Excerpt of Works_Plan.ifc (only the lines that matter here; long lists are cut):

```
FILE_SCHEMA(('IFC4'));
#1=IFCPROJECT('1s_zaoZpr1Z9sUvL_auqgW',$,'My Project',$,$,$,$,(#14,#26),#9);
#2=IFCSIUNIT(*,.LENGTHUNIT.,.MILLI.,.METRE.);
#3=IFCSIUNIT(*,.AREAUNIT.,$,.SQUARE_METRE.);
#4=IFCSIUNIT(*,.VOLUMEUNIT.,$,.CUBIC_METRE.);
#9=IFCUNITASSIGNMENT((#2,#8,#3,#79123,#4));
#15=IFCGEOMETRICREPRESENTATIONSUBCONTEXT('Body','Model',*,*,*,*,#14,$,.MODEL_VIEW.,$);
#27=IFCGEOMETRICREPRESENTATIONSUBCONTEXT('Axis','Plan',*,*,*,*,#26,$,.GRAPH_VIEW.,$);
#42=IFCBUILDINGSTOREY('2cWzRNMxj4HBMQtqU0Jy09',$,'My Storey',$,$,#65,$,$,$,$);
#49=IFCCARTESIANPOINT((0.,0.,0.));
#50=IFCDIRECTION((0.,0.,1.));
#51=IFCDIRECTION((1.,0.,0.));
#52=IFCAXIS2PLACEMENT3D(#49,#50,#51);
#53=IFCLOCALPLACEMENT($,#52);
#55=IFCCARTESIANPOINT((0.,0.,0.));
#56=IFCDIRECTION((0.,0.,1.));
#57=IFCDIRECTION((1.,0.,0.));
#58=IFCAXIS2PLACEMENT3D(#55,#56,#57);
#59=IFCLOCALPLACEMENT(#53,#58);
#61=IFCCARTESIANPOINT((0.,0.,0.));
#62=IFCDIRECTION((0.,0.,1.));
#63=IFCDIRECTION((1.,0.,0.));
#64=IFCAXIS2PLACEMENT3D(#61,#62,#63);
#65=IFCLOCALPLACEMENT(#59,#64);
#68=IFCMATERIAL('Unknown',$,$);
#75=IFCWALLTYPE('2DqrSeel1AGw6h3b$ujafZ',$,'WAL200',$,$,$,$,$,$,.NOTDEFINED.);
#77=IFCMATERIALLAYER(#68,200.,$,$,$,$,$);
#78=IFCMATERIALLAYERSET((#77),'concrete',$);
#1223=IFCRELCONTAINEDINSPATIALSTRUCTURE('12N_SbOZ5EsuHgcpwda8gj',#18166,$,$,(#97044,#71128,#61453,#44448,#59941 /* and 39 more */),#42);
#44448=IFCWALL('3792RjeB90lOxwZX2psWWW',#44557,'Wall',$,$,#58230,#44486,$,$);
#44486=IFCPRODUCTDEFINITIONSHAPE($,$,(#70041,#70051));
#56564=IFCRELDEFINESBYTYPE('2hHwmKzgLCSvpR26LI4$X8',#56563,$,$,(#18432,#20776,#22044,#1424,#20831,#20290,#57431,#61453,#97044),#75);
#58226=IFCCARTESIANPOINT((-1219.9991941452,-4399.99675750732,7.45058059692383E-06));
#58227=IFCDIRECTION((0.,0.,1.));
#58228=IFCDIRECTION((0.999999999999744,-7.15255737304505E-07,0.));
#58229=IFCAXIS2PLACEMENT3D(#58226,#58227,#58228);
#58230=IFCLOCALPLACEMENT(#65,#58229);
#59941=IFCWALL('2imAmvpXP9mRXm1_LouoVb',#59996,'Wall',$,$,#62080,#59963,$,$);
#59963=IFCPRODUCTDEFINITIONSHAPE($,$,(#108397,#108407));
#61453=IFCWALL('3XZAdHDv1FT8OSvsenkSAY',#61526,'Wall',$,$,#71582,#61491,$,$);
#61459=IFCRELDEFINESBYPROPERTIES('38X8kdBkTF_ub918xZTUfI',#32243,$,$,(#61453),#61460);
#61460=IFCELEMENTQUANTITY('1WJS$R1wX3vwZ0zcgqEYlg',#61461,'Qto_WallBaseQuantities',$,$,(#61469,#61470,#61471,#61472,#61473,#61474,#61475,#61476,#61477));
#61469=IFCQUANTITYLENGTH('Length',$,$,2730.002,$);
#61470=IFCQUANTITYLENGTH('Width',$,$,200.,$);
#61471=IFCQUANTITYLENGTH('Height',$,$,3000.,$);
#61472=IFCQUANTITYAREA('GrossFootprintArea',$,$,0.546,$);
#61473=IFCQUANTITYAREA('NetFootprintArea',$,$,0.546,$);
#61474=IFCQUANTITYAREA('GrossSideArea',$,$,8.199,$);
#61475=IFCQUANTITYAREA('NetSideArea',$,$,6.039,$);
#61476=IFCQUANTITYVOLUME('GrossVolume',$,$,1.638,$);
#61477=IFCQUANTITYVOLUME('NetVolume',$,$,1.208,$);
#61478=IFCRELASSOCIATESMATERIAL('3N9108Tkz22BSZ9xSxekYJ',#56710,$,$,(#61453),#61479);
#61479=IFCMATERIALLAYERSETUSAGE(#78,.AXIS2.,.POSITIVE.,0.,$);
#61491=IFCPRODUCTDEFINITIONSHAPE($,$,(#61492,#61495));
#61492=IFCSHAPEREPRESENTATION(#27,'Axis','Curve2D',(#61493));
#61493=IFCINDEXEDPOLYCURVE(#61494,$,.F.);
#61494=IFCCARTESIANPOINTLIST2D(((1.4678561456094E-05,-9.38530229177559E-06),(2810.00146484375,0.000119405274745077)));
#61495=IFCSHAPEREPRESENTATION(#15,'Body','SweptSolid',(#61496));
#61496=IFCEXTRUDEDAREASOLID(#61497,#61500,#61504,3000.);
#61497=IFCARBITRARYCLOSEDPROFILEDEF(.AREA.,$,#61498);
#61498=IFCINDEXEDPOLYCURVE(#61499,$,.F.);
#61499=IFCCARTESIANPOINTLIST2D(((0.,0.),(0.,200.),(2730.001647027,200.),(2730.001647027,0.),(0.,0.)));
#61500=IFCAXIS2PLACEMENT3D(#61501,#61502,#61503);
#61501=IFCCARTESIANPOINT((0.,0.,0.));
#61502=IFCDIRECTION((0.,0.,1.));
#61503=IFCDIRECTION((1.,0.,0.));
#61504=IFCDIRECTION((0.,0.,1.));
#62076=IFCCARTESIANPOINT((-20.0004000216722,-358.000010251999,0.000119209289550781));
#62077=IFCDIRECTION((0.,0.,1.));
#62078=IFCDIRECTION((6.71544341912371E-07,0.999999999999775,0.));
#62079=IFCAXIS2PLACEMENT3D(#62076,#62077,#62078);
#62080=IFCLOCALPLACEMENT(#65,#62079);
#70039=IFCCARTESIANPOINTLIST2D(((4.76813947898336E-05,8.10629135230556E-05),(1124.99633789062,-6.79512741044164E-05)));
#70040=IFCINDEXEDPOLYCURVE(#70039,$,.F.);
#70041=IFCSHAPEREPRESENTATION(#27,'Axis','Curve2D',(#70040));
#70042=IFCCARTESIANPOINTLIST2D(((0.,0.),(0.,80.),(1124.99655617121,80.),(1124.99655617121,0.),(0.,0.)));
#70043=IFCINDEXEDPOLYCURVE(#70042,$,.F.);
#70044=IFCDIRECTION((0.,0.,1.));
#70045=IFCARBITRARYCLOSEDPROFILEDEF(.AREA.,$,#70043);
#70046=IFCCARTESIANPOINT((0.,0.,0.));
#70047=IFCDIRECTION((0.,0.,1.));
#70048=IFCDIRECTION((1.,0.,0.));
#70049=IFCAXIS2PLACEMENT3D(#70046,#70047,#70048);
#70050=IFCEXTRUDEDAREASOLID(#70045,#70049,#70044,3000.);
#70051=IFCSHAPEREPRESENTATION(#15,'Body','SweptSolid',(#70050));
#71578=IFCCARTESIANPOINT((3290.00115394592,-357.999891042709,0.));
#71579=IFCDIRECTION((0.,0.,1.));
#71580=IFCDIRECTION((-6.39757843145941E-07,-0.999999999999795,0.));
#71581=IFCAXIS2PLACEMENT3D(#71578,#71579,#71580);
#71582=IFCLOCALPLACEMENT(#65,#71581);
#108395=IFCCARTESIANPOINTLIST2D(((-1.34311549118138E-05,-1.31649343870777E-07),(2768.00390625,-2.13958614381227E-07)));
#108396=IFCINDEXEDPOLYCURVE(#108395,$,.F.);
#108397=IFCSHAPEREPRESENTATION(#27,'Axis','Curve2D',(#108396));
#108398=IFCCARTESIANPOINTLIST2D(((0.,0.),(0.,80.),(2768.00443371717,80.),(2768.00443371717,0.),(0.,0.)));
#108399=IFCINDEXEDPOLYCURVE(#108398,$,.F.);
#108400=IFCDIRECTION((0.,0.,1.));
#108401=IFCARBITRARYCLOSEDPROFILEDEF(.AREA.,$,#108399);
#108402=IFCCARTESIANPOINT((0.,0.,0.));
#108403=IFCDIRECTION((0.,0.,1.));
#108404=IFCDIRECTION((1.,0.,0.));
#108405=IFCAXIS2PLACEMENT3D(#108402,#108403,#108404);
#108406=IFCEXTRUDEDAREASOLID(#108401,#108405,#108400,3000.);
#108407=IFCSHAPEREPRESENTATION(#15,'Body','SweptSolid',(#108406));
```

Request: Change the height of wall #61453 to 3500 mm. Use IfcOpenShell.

```python
import ifcopenshell
import ifcopenshell.api.pset
import ifcopenshell.geom
import ifcopenshell.util.element
import ifcopenshell.util.representation
import ifcopenshell.util.shape
import ifcopenshell.util.unit

model = ifcopenshell.open("Works_Plan.ifc")
unit_scale = ifcopenshell.util.unit.calculate_unit_scale(model)
area_scale = ifcopenshell.util.unit.calculate_unit_scale(model, "AREAUNIT")
volume_scale = ifcopenshell.util.unit.calculate_unit_scale(model, "VOLUMEUNIT")
settings = ifcopenshell.geom.settings()


def volume(element):
    """Net volume in cubic metres, openings subtracted."""
    shape = ifcopenshell.geom.create_shape(settings, element)
    return ifcopenshell.util.shape.get_volume(shape.geometry)


wall = model.by_guid("3XZAdHDv1FT8OSvsenkSAY")
before = volume(wall)

body = ifcopenshell.util.representation.get_representation(wall, "Model", "Body")
solid = body.Items[0]
old_height = solid.Depth
solid.Depth = 3.5 / unit_scale
after = volume(wall)
thickness = 0.2  # wall thickness in metres

# Update the stored height, areas and volumes.
qto = model.by_id(ifcopenshell.util.element.get_pset(wall, "Qto_WallBaseQuantities", should_inherit=False)["id"])
ifcopenshell.api.pset.edit_qto(model, qto=qto, properties={
    "Height": solid.Depth,
    "GrossSideArea": ifcopenshell.util.element.get_pset(wall, "Qto_WallBaseQuantities", "GrossSideArea") * solid.Depth / old_height,
    "NetSideArea": after / thickness / area_scale,
    "GrossVolume": ifcopenshell.util.element.get_pset(wall, "Qto_WallBaseQuantities", "GrossVolume") * solid.Depth / old_height,
    "NetVolume": after / volume_scale,
})

print(f"height {old_height:g} -> {solid.Depth:g}, volume {before:.3f} -> {after:.3f} m3")

model.write("Works_Plan_rev.ifc")
```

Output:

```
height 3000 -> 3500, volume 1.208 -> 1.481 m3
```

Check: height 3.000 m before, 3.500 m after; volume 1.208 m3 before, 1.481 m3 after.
